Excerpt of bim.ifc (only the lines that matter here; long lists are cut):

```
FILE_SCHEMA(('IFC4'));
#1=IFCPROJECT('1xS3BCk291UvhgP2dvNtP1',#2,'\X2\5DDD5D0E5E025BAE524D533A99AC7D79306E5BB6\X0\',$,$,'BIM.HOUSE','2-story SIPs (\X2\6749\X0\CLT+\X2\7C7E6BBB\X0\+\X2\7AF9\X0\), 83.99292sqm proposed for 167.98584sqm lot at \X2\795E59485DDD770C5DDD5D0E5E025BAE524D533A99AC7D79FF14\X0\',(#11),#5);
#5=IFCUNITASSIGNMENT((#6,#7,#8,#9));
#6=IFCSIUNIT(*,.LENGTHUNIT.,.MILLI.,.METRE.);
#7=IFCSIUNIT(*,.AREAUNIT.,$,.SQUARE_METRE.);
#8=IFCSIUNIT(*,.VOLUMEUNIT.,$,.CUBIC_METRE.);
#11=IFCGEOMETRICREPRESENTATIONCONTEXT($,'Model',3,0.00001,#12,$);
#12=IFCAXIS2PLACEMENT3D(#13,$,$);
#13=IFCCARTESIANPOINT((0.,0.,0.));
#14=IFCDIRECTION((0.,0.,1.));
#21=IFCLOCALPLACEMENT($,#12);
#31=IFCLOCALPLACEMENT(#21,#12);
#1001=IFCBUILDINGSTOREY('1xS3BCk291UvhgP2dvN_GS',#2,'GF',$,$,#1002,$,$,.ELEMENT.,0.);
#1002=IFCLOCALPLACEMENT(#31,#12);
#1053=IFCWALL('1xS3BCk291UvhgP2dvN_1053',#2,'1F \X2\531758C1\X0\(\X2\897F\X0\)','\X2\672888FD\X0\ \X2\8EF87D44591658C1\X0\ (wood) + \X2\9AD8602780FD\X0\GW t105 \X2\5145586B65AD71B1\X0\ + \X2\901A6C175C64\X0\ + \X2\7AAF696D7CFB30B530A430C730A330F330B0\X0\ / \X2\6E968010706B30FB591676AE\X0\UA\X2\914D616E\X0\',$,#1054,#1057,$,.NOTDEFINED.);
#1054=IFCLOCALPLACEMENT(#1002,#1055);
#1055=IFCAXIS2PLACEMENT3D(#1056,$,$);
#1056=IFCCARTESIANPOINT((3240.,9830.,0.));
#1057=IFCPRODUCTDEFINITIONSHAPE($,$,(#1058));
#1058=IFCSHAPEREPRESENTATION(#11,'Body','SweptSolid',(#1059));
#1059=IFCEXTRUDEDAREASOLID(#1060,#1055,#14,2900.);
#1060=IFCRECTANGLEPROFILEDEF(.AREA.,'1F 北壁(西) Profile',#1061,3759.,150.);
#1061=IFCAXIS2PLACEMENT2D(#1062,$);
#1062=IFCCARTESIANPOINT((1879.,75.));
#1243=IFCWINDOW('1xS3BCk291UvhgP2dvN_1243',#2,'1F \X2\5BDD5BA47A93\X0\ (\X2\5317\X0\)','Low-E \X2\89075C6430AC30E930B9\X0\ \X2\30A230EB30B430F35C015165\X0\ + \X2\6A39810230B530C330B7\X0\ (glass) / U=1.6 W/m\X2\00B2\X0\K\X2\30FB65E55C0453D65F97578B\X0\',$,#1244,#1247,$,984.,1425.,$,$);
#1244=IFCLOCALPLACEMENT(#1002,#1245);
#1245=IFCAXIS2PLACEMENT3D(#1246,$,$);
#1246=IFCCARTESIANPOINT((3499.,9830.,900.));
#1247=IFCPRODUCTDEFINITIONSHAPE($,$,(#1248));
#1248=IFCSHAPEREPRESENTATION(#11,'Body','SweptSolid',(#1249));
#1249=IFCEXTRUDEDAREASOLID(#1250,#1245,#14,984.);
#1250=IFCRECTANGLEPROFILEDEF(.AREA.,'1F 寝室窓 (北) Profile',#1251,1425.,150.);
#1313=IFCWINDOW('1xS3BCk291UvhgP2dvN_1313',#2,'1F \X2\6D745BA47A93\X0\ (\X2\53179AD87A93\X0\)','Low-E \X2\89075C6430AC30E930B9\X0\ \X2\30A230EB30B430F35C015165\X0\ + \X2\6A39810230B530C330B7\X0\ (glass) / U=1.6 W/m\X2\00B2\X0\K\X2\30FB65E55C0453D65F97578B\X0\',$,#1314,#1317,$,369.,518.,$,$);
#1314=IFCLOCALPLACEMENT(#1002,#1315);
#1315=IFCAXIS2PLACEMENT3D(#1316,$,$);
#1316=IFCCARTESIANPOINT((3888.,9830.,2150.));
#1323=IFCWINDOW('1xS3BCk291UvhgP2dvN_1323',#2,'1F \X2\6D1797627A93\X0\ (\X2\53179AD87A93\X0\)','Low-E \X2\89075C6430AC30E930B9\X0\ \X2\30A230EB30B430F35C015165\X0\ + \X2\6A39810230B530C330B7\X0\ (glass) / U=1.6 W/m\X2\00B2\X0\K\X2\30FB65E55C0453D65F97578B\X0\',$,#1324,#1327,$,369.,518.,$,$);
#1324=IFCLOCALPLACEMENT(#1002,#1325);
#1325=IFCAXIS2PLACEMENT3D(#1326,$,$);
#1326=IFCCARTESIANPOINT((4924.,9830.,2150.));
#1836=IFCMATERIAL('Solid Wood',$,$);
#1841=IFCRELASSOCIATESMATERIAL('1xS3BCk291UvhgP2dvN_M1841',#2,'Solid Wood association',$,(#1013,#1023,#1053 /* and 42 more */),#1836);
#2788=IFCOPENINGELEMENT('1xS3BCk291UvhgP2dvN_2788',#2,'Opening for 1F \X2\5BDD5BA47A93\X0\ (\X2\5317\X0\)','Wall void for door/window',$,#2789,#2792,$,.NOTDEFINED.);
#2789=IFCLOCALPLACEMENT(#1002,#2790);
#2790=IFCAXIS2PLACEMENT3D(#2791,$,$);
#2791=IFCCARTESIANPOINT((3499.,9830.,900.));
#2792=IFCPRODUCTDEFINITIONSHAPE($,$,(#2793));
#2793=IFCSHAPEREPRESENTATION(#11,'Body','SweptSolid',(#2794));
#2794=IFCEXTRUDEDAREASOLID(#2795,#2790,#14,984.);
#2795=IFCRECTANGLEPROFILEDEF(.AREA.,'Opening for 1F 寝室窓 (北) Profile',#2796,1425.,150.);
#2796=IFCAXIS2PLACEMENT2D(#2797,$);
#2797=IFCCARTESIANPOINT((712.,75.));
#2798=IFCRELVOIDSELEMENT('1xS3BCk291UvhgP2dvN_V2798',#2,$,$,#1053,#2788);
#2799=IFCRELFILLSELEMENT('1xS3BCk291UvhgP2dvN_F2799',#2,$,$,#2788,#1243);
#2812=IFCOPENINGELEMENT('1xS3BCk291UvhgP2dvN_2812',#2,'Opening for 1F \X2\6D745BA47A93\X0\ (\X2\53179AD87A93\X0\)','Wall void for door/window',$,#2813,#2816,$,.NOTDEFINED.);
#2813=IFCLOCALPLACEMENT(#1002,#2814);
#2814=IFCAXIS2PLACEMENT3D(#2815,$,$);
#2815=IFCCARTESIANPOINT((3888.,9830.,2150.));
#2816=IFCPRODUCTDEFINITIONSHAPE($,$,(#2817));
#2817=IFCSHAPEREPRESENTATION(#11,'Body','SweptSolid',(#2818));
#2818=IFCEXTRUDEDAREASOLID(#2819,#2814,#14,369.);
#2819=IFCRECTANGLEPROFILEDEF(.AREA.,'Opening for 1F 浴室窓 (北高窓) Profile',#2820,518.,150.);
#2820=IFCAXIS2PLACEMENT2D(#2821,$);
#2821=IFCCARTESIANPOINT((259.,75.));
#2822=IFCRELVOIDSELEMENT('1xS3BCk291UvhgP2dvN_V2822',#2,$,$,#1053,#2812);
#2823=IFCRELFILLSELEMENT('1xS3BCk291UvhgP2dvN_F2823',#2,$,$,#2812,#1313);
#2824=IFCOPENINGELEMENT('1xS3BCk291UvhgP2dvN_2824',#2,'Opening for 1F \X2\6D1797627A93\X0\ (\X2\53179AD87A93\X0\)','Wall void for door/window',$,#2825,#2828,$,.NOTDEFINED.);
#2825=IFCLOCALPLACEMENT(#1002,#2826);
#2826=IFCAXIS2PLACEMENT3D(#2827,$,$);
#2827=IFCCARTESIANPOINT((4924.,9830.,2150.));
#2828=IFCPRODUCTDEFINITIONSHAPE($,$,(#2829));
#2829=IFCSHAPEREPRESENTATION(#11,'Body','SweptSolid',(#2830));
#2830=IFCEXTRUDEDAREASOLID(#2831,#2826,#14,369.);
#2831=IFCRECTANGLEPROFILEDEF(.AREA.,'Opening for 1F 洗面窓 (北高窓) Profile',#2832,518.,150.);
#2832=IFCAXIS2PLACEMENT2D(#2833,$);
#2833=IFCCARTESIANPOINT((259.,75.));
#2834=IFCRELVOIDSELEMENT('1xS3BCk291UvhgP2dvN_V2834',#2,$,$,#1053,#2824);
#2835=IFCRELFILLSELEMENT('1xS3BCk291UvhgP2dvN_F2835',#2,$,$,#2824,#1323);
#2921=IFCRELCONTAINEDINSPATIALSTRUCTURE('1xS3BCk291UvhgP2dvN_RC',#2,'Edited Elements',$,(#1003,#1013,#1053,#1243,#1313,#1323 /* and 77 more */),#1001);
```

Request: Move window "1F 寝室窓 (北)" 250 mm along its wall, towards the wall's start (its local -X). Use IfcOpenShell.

```python
import ifcopenshell
import ifcopenshell.api.geometry
import ifcopenshell.util.placement
import ifcopenshell.util.unit

model = ifcopenshell.open("bim.ifc")
unit_scale = ifcopenshell.util.unit.calculate_unit_scale(model)

window = model.by_guid("1xS3BCk291UvhgP2dvN_1243")
opening = window.FillsVoids[0].RelatingOpeningElement
wall = opening.VoidsElements[0].RelatingBuildingElement

wall_matrix = ifcopenshell.util.placement.get_local_placement(wall.ObjectPlacement)
shift = wall_matrix[:3, 0] * -0.25 / unit_scale
before = ifcopenshell.util.placement.get_local_placement(window.ObjectPlacement)[:3, 3].copy()

# The window is not placed relative to its opening, so move both.
for product in (opening, window):
    matrix = ifcopenshell.util.placement.get_local_placement(product.ObjectPlacement)
    matrix[:3, 3] += shift
    ifcopenshell.api.geometry.edit_object_placement(model, product=product, matrix=matrix, is_si=False)

after = ifcopenshell.util.placement.get_local_placement(window.ObjectPlacement)[:3, 3]
print("window moved by", (after - before).round(3) + 0.0)

model.write("bim_v2.ifc")
```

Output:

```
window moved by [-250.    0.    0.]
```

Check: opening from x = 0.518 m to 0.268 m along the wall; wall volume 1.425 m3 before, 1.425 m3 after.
